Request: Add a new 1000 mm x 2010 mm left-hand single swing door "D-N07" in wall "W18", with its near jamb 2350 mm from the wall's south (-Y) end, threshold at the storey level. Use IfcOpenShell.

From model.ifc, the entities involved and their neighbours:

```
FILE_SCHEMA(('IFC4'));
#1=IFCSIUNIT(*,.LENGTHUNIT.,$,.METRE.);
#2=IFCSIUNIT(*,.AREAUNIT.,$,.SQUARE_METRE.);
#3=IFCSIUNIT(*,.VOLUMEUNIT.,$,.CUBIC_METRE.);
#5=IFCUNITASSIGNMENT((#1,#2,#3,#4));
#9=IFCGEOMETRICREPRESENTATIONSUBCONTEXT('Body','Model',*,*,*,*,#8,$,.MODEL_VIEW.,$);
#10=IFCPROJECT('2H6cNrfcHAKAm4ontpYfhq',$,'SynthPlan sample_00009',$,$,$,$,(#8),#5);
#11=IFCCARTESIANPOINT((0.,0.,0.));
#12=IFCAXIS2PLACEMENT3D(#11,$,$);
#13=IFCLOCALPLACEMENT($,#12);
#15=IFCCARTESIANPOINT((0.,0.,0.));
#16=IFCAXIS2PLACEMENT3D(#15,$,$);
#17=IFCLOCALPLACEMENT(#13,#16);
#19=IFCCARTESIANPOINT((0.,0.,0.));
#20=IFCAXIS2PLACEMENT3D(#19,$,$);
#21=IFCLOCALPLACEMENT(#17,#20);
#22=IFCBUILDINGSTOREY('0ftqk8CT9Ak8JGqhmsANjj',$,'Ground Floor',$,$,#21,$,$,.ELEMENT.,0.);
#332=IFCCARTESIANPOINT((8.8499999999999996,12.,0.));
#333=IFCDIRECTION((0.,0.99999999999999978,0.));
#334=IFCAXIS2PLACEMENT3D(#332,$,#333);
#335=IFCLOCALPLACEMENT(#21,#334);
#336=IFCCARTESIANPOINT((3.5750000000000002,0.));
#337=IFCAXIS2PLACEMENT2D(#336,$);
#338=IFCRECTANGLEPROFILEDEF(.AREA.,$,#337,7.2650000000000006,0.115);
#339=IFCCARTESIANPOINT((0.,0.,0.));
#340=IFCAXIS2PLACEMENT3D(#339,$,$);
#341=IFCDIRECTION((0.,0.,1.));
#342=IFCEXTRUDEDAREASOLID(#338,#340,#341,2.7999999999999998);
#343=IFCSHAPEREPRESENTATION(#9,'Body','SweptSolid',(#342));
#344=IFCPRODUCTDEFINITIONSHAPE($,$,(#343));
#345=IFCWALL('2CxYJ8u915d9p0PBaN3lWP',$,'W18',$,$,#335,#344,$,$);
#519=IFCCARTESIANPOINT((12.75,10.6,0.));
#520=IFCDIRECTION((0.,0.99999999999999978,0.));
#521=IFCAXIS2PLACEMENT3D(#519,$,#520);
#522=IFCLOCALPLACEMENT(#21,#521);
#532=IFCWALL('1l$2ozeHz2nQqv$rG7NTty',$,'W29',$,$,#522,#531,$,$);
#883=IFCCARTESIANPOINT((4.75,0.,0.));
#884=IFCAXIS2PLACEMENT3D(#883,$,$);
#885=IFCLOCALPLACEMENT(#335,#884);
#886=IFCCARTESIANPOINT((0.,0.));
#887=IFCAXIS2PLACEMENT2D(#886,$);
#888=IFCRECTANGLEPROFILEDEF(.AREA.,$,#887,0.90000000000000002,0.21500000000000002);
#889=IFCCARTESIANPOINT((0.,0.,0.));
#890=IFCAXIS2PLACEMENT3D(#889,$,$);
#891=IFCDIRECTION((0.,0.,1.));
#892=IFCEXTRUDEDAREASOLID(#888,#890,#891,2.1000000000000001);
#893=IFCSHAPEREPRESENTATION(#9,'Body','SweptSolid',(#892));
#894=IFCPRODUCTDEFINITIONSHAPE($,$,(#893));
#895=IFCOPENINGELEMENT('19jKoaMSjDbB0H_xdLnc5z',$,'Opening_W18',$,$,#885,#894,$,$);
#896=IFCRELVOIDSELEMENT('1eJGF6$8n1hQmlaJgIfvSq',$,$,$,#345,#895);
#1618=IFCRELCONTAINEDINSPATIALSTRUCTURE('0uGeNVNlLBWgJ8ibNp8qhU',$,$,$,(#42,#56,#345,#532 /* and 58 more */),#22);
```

```python
import numpy as np
import ifcopenshell
import ifcopenshell.api.feature
import ifcopenshell.api.geometry
import ifcopenshell.api.root
import ifcopenshell.api.spatial
import ifcopenshell.geom
import ifcopenshell.util.element
import ifcopenshell.util.placement
import ifcopenshell.util.representation
import ifcopenshell.util.shape
import ifcopenshell.util.unit

model = ifcopenshell.open("model.ifc")
unit_scale = ifcopenshell.util.unit.calculate_unit_scale(model)
settings = ifcopenshell.geom.settings()


def volume(element):
    """Net volume in cubic metres, openings subtracted."""
    shape = ifcopenshell.geom.create_shape(settings, element)
    return ifcopenshell.util.shape.get_volume(shape.geometry)


wall = model.by_guid("2CxYJ8u915d9p0PBaN3lWP")
storey = ifcopenshell.util.element.get_container(wall, ifc_class="IfcBuildingStorey")
context = ifcopenshell.util.representation.get_context(model, "Model", "Body", "MODEL_VIEW")
before = volume(wall)

width, height, from_end, sill = 1, 2.01, 2.35, 0.0  # metres

# The wall runs along its own X axis, and the end named is its -X end.
wall_shape = ifcopenshell.geom.create_shape(settings, wall)
x, y, z = ifcopenshell.util.shape.get_vertices(wall_shape.geometry).T
start = x.min() + from_end
face, thickness = float(y.min()), float(y.max() - y.min())
wall_matrix = ifcopenshell.util.placement.get_local_placement(wall.ObjectPlacement)
level = ifcopenshell.util.placement.get_local_placement(storey.ObjectPlacement)[2, 3]


def in_wall(x, y):
    """Placement at x, y metres in the wall's axes, at sill height."""
    matrix = wall_matrix.copy()
    matrix[:, 3] = wall_matrix @ np.array([x / unit_scale, y / unit_scale, 0.0, 1.0])
    matrix[2, 3] = level + sill / unit_scale
    return matrix


# Opening: a box that overshoots both wall faces by 50 mm.
opening = ifcopenshell.api.root.create_entity(model, ifc_class="IfcOpeningElement", predefined_type="OPENING")
box = ifcopenshell.api.geometry.add_wall_representation(
    model, context=context, length=width, height=height, thickness=thickness + 0.1
)
ifcopenshell.api.geometry.assign_representation(model, product=opening, representation=box)
ifcopenshell.api.geometry.edit_object_placement(model, product=opening, matrix=in_wall(start, face - 0.05), is_si=False)
ifcopenshell.api.feature.add_feature(model, feature=opening, element=wall)

door = ifcopenshell.api.root.create_entity(model, ifc_class="IfcDoor", name="D-N07", predefined_type="DOOR")
door.OverallWidth, door.OverallHeight = width / unit_scale, height / unit_scale
door.OperationType = "SINGLE_SWING_LEFT"
body = ifcopenshell.api.geometry.add_door_representation(
    model,
    context=context,
    overall_width=door.OverallWidth,
    overall_height=door.OverallHeight,
    operation_type="SINGLE_SWING_LEFT",
    lining_properties={"LiningDepth": thickness / unit_scale, "ThresholdDepth": thickness / unit_scale},
)
ifcopenshell.api.geometry.assign_representation(model, product=door, representation=body)
ifcopenshell.api.spatial.assign_container(model, products=[door], relating_structure=storey)
ifcopenshell.api.feature.add_filling(model, opening=opening, element=door)

# The lining spans the wall, so the door starts at the wall face.
ifcopenshell.api.geometry.edit_object_placement(model, product=door, matrix=in_wall(start, face), is_si=False)

after = volume(wall)

print(f"wall volume {before:.3f} -> {after:.3f} m3")

model.write("model_rev.ifc")
```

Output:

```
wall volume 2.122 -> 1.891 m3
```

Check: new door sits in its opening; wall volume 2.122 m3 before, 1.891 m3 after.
